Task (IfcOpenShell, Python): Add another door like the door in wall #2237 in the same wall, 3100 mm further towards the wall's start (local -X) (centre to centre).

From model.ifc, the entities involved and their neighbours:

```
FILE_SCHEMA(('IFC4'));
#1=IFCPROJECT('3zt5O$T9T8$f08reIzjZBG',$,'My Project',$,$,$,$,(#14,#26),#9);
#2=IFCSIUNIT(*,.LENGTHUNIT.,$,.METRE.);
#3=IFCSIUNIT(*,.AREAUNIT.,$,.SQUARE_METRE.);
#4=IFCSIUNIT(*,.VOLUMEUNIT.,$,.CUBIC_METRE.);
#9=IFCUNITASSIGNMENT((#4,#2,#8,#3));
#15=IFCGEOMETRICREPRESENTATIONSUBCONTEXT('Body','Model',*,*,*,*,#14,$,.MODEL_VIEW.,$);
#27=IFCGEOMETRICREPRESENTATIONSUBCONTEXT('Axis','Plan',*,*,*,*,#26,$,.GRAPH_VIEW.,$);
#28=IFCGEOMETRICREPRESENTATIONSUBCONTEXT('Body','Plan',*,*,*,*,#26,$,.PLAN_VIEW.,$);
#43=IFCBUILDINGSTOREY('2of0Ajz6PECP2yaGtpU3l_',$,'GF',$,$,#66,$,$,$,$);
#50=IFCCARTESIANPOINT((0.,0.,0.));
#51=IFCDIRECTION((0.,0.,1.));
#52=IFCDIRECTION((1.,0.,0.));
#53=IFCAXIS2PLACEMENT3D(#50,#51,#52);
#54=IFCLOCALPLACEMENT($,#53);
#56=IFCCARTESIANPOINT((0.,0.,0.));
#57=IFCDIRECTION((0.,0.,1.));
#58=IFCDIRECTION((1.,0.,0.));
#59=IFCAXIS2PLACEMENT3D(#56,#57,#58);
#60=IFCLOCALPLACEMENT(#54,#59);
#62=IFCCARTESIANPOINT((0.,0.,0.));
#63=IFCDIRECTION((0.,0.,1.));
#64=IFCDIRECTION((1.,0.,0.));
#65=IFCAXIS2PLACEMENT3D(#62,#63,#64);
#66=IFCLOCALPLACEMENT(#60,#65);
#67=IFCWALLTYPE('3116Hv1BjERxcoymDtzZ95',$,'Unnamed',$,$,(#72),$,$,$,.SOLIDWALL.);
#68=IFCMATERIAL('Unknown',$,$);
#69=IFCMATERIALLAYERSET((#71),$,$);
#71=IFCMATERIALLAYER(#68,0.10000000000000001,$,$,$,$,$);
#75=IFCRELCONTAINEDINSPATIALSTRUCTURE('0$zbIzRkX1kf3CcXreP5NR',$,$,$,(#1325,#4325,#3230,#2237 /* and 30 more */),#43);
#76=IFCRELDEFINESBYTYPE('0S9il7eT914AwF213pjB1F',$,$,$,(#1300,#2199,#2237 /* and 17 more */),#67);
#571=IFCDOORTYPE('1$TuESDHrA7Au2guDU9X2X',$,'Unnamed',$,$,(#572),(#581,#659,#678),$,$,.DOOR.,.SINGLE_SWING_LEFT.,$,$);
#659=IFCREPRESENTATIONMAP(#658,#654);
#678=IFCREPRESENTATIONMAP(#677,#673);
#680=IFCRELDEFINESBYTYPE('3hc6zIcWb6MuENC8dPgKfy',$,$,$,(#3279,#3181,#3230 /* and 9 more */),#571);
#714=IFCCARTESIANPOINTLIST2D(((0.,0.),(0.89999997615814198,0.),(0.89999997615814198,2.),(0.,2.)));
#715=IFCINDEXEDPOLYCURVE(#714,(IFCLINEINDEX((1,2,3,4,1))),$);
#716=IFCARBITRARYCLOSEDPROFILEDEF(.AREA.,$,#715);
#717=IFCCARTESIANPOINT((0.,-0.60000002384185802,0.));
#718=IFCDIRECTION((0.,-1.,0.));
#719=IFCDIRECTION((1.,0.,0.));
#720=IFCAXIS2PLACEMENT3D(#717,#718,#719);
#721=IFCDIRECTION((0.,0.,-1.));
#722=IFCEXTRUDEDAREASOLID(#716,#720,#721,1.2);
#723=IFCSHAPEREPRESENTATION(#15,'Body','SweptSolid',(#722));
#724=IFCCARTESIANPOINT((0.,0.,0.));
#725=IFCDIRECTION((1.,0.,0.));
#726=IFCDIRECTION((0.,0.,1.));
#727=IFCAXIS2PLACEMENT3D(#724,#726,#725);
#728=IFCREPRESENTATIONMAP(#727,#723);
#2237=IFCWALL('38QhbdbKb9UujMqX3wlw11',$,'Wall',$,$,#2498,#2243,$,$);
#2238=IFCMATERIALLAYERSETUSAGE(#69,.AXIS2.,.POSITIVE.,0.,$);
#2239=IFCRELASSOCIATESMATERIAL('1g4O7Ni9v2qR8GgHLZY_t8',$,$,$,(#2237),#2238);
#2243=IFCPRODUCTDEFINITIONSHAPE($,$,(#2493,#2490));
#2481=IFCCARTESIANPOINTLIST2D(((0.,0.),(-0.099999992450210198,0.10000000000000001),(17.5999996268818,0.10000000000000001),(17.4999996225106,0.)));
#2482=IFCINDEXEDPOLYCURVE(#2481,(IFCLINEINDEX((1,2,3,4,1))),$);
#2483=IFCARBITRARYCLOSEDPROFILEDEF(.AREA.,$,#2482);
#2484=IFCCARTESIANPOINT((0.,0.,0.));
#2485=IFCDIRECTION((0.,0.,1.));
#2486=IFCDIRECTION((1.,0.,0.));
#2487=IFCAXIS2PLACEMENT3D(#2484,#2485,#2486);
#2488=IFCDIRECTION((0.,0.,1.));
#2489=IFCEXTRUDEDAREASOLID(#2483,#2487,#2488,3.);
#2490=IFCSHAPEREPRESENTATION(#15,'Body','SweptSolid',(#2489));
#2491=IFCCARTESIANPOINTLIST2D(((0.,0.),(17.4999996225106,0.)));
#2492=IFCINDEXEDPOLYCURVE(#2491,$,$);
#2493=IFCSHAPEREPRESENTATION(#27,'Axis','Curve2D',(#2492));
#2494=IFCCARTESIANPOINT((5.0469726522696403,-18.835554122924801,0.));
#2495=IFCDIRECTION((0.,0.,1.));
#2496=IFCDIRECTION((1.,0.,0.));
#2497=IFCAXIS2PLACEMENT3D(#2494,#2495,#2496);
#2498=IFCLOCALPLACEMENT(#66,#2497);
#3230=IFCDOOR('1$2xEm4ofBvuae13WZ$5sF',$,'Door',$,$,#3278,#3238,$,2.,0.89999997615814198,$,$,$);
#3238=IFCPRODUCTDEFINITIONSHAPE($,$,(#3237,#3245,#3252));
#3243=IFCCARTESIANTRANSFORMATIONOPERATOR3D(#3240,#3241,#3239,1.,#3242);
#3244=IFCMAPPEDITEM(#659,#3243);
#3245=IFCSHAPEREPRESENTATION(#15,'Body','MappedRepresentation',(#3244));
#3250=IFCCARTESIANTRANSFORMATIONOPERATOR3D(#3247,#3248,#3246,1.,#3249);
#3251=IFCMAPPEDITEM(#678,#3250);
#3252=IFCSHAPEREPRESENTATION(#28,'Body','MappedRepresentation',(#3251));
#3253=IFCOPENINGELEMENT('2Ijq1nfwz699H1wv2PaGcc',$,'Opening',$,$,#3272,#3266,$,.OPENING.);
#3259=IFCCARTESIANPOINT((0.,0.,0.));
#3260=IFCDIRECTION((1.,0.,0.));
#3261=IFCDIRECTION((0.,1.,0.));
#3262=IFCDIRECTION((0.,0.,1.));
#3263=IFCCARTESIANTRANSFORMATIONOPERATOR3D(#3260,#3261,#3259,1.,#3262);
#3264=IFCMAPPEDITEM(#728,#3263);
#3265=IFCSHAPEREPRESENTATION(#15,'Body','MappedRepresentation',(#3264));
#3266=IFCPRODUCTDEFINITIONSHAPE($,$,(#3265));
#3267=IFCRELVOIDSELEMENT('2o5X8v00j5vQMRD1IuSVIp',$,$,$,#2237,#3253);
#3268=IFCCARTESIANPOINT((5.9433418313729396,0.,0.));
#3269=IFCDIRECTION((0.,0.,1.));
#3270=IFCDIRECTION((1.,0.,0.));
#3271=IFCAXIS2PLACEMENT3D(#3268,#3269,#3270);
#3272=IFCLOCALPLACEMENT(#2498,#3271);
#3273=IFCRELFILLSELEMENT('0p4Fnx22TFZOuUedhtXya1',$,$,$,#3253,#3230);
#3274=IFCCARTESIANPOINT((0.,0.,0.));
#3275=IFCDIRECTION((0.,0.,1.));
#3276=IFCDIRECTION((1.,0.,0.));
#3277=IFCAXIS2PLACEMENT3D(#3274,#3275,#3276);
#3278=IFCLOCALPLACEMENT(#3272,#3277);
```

```python
import ifcopenshell
import ifcopenshell.api.feature
import ifcopenshell.api.geometry
import ifcopenshell.api.root
import ifcopenshell.geom
import ifcopenshell.util.element
import ifcopenshell.util.placement
import ifcopenshell.util.shape
import ifcopenshell.util.unit

model = ifcopenshell.open("model.ifc")
unit_scale = ifcopenshell.util.unit.calculate_unit_scale(model)
settings = ifcopenshell.geom.settings()


def volume(element):
    """Net volume in cubic metres, openings subtracted."""
    shape = ifcopenshell.geom.create_shape(settings, element)
    return ifcopenshell.util.shape.get_volume(shape.geometry)


door = model.by_id(3230)
opening = door.FillsVoids[0].RelatingOpeningElement
wall = opening.VoidsElements[0].RelatingBuildingElement
before = volume(wall)
shift = ifcopenshell.util.placement.get_local_placement(wall.ObjectPlacement)[:3, 0] * -3.1 / unit_scale

# copy_class copies the void relationship, type, container and properties, but no geometry.
new_opening = ifcopenshell.api.root.copy_class(model, product=opening)
new_opening.Representation = ifcopenshell.util.element.copy_deep(
    model, opening.Representation, exclude=["IfcGeometricRepresentationContext", "IfcRepresentationMap"]
)
new_door = ifcopenshell.api.root.copy_class(model, product=door)
new_door.Representation = ifcopenshell.util.element.copy_deep(
    model, door.Representation, exclude=["IfcGeometricRepresentationContext", "IfcRepresentationMap"]
)
ifcopenshell.api.feature.add_filling(model, opening=new_opening, element=new_door)

for old, new in ((opening, new_opening), (door, new_door)):
    matrix = ifcopenshell.util.placement.get_local_placement(old.ObjectPlacement)
    matrix[:3, 3] += shift
    ifcopenshell.api.geometry.edit_object_placement(model, product=new, matrix=matrix, is_si=False)

after = volume(wall)

print(f"wall volume {before:.3f} -> {after:.3f} m3")

model.write("model_edited.ifc")
```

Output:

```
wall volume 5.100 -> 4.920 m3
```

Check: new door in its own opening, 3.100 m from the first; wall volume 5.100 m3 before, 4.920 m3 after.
